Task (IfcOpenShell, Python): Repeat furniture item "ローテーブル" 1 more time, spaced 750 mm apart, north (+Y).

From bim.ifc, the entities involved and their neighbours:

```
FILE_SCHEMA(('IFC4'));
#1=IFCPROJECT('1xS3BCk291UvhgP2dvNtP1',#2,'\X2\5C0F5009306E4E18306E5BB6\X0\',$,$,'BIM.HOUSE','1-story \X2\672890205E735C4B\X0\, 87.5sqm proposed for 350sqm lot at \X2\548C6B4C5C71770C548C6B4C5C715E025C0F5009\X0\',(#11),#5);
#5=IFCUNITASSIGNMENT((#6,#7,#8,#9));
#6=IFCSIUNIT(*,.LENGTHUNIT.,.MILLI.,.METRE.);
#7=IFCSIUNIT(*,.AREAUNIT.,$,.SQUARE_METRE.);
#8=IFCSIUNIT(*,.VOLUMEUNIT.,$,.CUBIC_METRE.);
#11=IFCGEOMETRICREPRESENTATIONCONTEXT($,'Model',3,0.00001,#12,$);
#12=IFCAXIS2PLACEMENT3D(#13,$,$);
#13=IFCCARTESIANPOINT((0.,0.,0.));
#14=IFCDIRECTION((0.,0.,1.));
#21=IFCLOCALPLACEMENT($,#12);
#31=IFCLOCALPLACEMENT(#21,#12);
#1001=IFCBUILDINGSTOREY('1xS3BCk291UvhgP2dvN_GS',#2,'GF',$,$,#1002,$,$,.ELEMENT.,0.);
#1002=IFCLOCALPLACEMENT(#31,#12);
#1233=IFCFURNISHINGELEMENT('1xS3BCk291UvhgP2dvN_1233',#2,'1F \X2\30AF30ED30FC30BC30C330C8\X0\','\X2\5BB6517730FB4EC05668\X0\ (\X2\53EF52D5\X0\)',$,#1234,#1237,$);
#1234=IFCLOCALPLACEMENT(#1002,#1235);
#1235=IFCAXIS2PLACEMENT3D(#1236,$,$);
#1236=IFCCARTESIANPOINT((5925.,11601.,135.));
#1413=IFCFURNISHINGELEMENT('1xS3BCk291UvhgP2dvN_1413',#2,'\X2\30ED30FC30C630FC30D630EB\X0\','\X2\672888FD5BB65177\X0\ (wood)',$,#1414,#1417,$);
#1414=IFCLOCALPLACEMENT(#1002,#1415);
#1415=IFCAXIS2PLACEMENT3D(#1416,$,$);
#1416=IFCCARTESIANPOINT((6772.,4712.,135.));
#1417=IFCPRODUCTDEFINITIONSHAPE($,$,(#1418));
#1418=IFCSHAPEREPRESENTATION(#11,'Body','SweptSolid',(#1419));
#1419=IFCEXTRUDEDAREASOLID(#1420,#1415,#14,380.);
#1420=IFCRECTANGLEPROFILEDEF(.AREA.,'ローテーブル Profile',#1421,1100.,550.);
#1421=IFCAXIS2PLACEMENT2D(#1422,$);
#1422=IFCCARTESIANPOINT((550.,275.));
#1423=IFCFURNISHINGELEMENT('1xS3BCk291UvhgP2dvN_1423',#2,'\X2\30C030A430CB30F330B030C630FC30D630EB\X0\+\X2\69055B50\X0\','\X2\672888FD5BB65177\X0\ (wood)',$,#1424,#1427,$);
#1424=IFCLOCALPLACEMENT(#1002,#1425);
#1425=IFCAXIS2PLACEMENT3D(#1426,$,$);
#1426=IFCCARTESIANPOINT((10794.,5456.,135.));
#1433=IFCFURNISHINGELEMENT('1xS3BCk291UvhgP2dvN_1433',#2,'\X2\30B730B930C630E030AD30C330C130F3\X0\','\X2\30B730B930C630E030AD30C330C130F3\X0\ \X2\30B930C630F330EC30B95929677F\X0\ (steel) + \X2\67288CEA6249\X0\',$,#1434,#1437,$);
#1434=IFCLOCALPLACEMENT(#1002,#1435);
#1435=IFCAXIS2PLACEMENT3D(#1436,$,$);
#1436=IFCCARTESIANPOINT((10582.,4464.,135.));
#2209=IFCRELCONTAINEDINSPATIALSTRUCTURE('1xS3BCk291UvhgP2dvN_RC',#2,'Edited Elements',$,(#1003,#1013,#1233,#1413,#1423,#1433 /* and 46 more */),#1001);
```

```python
import numpy as np
import ifcopenshell
import ifcopenshell.api.geometry
import ifcopenshell.api.root
import ifcopenshell.util.element
import ifcopenshell.util.placement

model = ifcopenshell.open("bim.ifc")


def reuse_history(source, copy):
    """copy_class also copies each property set's owner history, people and application; keep the originals."""
    for rel in copy.IsDefinedBy:
        if rel.is_a("IfcRelDefinesByProperties") and (history := rel.RelatingPropertyDefinition.OwnerHistory):
            rel.RelatingPropertyDefinition.OwnerHistory = source.OwnerHistory
            ifcopenshell.util.element.remove_deep2(model, history)


source = model.by_id(1413)
base = ifcopenshell.util.placement.get_local_placement(source.ObjectPlacement)
step = np.array([0.0, 1.0, 0.0]) * 750.0

for i in range(1, 2):
    copy = ifcopenshell.api.root.copy_class(model, product=source)
    copy.Representation = ifcopenshell.util.element.copy_deep(
        model, source.Representation, exclude=["IfcGeometricRepresentationContext", "IfcRepresentationMap"]
    )
    reuse_history(source, copy)
    matrix = base.copy()
    matrix[:3, 3] += i * step
    print("added at", matrix[:3, 3].round(3) + 0.0)
    ifcopenshell.api.geometry.edit_object_placement(model, product=copy, matrix=matrix, is_si=False)

model.write("bim_v2.ifc")
```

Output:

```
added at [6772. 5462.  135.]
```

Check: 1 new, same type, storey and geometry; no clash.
